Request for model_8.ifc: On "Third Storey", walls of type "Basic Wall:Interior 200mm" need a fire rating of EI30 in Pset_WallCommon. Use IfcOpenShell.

First a look at what the model holds.

```python
import ifcopenshell
import ifcopenshell.util.element

model = ifcopenshell.open("model_8.ifc")
print(model.schema)
storey = next(s for s in model.by_type("IfcBuildingStorey") if s.Name == "Third Storey")
walls = [e for e in ifcopenshell.util.element.get_decomposition(storey) if e.is_a("IfcWall")]
seen = {}
for e in walls:
    element_type = ifcopenshell.util.element.get_type(e)
    key = (element_type.Name if element_type != e and element_type else None, ifcopenshell.util.element.get_pset(e, "Pset_WallCommon", "FireRating"))
    seen[key] = seen.get(key, 0) + 1
for (name, value), count in sorted(seen.items(), key=str):
    print(count, "x", name, "|", value)
```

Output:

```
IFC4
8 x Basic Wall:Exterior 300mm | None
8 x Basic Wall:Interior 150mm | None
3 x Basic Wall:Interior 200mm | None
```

```python
import ifcopenshell
import ifcopenshell.api.pset
import ifcopenshell.util.element

model = ifcopenshell.open("model_8.ifc")

storey = next(s for s in model.by_type("IfcBuildingStorey") if s.Name == "Third Storey")
walls = [e for e in ifcopenshell.util.element.get_decomposition(storey) if e.is_a("IfcWall")]

count = 0
for e in walls:
    element_type = ifcopenshell.util.element.get_type(e)
    if element_type in (None, e) or element_type.Name != "Basic Wall:Interior 200mm":
        continue
    # add_pset returns the element's existing set when there is one.
    pset = ifcopenshell.api.pset.add_pset(model, product=e, name="Pset_WallCommon")
    ifcopenshell.api.pset.edit_pset(model, pset=pset, properties={"FireRating": "EI30"})
    count += 1

print(count, "walls updated")

model.write("model_8-out.ifc")
```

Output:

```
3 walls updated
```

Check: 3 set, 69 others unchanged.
